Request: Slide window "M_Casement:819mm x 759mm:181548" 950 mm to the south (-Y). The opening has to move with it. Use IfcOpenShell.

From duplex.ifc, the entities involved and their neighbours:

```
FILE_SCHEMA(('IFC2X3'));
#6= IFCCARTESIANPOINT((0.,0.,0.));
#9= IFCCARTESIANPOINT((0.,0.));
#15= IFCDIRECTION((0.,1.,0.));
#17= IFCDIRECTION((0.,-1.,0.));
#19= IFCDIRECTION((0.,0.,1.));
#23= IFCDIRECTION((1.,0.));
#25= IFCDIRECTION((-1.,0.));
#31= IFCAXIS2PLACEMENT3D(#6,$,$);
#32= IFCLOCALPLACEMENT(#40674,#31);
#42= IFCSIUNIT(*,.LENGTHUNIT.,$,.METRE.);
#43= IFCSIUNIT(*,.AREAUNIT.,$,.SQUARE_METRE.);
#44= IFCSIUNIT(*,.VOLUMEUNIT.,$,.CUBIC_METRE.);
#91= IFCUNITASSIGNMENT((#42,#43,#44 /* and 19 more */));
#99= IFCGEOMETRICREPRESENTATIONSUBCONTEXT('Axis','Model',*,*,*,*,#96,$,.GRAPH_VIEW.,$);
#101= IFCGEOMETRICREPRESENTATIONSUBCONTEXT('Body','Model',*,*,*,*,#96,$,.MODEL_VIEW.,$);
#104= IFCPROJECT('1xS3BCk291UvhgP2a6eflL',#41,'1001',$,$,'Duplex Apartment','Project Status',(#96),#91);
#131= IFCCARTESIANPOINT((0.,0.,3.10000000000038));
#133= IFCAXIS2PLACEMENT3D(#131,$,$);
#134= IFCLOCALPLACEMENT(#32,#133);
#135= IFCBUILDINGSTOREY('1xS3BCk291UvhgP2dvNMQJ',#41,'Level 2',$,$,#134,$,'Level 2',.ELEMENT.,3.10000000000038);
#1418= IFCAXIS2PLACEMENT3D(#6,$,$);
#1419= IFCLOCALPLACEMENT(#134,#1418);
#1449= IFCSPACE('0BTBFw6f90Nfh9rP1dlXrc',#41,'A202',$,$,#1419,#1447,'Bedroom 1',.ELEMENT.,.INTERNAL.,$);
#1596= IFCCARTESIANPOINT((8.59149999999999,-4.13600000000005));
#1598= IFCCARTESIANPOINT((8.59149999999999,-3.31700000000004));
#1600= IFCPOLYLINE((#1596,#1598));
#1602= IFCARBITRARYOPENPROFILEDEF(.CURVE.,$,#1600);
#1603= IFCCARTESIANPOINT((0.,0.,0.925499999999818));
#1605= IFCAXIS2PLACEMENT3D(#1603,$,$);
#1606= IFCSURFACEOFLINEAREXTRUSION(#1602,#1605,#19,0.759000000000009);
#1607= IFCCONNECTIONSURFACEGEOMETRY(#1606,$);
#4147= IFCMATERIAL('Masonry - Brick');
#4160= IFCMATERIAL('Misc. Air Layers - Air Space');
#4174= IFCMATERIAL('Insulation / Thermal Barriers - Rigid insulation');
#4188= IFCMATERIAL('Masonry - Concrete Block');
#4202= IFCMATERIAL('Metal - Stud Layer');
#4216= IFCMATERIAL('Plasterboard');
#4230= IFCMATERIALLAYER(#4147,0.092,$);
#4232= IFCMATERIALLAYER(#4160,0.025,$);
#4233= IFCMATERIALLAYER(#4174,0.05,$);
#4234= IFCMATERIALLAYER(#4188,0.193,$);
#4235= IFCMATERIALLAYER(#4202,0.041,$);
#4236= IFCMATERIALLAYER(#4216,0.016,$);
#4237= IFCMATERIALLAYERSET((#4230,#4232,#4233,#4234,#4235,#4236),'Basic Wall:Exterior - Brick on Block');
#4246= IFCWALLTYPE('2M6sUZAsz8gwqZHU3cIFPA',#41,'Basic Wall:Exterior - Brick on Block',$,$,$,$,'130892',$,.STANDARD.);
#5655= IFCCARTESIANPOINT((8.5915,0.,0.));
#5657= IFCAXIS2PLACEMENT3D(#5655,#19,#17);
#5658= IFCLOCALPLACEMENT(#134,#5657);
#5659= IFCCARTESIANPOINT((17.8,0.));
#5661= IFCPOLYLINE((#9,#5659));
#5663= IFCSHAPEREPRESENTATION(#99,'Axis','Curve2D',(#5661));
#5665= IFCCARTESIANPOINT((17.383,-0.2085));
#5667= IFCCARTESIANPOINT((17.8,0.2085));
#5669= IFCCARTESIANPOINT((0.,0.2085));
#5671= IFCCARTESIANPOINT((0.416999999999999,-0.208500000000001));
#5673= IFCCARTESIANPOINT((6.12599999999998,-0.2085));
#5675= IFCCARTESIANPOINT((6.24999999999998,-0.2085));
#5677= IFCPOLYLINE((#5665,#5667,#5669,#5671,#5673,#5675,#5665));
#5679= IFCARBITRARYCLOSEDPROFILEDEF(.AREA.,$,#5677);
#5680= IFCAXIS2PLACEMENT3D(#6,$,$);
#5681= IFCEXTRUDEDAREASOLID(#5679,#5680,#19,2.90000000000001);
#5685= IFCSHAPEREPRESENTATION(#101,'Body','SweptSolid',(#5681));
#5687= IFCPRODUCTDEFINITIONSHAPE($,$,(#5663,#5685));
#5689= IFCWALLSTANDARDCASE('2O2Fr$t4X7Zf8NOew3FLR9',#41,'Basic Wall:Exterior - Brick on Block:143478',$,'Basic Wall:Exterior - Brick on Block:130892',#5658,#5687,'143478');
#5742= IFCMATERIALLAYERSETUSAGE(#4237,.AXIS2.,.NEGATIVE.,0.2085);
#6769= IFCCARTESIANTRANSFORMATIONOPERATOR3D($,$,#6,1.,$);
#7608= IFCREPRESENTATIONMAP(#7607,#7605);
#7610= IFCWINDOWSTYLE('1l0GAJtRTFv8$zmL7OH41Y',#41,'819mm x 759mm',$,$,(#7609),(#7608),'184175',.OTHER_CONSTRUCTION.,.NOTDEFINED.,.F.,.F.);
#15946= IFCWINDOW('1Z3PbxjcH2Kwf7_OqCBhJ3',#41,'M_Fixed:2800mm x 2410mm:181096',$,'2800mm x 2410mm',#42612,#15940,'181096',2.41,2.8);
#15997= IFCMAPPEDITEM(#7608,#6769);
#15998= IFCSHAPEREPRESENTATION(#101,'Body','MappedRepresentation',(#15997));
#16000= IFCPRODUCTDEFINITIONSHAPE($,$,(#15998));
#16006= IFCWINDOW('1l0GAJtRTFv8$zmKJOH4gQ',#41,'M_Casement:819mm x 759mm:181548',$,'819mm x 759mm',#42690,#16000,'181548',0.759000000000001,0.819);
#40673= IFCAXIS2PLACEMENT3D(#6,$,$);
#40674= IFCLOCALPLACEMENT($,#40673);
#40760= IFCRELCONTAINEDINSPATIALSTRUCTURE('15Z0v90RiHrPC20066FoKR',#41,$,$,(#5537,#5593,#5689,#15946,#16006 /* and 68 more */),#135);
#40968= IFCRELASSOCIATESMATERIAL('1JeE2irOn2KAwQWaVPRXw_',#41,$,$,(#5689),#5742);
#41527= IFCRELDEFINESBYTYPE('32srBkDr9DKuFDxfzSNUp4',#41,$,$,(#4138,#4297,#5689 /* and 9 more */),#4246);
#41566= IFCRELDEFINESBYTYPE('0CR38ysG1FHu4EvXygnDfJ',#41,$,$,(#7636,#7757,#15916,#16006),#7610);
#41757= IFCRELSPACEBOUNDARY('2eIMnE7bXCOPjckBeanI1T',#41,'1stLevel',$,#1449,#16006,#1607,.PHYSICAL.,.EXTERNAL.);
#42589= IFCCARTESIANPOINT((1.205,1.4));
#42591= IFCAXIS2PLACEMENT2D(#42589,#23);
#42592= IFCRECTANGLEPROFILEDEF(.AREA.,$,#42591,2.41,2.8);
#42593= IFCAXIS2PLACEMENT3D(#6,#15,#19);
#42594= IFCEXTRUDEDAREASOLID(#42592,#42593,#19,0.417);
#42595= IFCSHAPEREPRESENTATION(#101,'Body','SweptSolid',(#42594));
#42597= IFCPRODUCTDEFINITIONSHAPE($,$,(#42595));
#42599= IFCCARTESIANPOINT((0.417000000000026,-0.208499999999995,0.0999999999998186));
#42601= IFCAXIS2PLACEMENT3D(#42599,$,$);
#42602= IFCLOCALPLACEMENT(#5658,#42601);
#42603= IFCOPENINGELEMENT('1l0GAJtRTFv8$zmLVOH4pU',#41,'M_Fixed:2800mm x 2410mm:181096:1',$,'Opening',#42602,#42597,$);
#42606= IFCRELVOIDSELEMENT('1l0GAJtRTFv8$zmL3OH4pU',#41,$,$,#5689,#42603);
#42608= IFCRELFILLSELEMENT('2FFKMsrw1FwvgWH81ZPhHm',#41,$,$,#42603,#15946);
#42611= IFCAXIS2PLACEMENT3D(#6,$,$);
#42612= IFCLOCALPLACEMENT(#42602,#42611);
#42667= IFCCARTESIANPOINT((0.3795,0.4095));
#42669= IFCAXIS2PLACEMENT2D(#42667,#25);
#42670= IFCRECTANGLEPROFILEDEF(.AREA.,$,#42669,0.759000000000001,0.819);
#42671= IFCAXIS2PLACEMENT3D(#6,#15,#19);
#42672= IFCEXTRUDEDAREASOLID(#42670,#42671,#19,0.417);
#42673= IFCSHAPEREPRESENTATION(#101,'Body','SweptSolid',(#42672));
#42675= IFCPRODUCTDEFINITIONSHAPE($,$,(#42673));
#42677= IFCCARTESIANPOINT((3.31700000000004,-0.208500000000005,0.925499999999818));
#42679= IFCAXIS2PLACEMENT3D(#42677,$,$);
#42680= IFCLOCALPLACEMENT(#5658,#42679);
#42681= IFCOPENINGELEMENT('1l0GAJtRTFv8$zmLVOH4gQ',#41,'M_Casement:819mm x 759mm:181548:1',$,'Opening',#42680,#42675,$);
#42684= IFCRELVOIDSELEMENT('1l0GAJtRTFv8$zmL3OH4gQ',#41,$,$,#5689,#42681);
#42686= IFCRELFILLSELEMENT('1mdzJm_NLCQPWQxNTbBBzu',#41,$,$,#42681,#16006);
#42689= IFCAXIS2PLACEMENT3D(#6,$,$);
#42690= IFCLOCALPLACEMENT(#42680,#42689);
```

```python
import numpy as np
import ifcopenshell
import ifcopenshell.api.geometry
import ifcopenshell.util.placement
import ifcopenshell.util.unit

model = ifcopenshell.open("duplex.ifc")
unit_scale = ifcopenshell.util.unit.calculate_unit_scale(model)

window = model.by_id(16006)
opening = window.FillsVoids[0].RelatingOpeningElement
wall = opening.VoidsElements[0].RelatingBuildingElement

wall_matrix = ifcopenshell.util.placement.get_local_placement(wall.ObjectPlacement)
shift = wall_matrix[:3, 0] * 0.95 / unit_scale
before = ifcopenshell.util.placement.get_local_placement(window.ObjectPlacement)[:3, 3].copy()

# The window is placed relative to its opening, so it follows when the opening moves.
matrix = ifcopenshell.util.placement.get_local_placement(opening.ObjectPlacement)
matrix[:3, 3] += shift
ifcopenshell.api.geometry.edit_object_placement(
    model, product=opening, matrix=matrix, is_si=False, should_transform_children=True
)

# Space boundary surfaces are stored in each space's coordinates; move them too.
for rel in window.ProvidesBoundaries:
    if not rel.ConnectionGeometry:
        continue
    surface = rel.ConnectionGeometry.SurfaceOnRelatingElement
    space_matrix = ifcopenshell.util.placement.get_local_placement(rel.RelatingSpace.ObjectPlacement)
    point = np.array(surface.Position.Location.Coordinates) + space_matrix[:3, :3].T @ shift
    surface.Position = model.createIfcAxis2Placement3D(
        model.createIfcCartesianPoint(point.tolist()), surface.Position.Axis, surface.Position.RefDirection
    )

after = ifcopenshell.util.placement.get_local_placement(window.ObjectPlacement)[:3, 3]
print("window moved by", (after - before).round(3) + 0.0)

model.write("duplex_edited.ifc")
```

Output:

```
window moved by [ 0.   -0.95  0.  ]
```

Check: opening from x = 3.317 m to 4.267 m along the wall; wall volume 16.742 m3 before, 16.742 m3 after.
